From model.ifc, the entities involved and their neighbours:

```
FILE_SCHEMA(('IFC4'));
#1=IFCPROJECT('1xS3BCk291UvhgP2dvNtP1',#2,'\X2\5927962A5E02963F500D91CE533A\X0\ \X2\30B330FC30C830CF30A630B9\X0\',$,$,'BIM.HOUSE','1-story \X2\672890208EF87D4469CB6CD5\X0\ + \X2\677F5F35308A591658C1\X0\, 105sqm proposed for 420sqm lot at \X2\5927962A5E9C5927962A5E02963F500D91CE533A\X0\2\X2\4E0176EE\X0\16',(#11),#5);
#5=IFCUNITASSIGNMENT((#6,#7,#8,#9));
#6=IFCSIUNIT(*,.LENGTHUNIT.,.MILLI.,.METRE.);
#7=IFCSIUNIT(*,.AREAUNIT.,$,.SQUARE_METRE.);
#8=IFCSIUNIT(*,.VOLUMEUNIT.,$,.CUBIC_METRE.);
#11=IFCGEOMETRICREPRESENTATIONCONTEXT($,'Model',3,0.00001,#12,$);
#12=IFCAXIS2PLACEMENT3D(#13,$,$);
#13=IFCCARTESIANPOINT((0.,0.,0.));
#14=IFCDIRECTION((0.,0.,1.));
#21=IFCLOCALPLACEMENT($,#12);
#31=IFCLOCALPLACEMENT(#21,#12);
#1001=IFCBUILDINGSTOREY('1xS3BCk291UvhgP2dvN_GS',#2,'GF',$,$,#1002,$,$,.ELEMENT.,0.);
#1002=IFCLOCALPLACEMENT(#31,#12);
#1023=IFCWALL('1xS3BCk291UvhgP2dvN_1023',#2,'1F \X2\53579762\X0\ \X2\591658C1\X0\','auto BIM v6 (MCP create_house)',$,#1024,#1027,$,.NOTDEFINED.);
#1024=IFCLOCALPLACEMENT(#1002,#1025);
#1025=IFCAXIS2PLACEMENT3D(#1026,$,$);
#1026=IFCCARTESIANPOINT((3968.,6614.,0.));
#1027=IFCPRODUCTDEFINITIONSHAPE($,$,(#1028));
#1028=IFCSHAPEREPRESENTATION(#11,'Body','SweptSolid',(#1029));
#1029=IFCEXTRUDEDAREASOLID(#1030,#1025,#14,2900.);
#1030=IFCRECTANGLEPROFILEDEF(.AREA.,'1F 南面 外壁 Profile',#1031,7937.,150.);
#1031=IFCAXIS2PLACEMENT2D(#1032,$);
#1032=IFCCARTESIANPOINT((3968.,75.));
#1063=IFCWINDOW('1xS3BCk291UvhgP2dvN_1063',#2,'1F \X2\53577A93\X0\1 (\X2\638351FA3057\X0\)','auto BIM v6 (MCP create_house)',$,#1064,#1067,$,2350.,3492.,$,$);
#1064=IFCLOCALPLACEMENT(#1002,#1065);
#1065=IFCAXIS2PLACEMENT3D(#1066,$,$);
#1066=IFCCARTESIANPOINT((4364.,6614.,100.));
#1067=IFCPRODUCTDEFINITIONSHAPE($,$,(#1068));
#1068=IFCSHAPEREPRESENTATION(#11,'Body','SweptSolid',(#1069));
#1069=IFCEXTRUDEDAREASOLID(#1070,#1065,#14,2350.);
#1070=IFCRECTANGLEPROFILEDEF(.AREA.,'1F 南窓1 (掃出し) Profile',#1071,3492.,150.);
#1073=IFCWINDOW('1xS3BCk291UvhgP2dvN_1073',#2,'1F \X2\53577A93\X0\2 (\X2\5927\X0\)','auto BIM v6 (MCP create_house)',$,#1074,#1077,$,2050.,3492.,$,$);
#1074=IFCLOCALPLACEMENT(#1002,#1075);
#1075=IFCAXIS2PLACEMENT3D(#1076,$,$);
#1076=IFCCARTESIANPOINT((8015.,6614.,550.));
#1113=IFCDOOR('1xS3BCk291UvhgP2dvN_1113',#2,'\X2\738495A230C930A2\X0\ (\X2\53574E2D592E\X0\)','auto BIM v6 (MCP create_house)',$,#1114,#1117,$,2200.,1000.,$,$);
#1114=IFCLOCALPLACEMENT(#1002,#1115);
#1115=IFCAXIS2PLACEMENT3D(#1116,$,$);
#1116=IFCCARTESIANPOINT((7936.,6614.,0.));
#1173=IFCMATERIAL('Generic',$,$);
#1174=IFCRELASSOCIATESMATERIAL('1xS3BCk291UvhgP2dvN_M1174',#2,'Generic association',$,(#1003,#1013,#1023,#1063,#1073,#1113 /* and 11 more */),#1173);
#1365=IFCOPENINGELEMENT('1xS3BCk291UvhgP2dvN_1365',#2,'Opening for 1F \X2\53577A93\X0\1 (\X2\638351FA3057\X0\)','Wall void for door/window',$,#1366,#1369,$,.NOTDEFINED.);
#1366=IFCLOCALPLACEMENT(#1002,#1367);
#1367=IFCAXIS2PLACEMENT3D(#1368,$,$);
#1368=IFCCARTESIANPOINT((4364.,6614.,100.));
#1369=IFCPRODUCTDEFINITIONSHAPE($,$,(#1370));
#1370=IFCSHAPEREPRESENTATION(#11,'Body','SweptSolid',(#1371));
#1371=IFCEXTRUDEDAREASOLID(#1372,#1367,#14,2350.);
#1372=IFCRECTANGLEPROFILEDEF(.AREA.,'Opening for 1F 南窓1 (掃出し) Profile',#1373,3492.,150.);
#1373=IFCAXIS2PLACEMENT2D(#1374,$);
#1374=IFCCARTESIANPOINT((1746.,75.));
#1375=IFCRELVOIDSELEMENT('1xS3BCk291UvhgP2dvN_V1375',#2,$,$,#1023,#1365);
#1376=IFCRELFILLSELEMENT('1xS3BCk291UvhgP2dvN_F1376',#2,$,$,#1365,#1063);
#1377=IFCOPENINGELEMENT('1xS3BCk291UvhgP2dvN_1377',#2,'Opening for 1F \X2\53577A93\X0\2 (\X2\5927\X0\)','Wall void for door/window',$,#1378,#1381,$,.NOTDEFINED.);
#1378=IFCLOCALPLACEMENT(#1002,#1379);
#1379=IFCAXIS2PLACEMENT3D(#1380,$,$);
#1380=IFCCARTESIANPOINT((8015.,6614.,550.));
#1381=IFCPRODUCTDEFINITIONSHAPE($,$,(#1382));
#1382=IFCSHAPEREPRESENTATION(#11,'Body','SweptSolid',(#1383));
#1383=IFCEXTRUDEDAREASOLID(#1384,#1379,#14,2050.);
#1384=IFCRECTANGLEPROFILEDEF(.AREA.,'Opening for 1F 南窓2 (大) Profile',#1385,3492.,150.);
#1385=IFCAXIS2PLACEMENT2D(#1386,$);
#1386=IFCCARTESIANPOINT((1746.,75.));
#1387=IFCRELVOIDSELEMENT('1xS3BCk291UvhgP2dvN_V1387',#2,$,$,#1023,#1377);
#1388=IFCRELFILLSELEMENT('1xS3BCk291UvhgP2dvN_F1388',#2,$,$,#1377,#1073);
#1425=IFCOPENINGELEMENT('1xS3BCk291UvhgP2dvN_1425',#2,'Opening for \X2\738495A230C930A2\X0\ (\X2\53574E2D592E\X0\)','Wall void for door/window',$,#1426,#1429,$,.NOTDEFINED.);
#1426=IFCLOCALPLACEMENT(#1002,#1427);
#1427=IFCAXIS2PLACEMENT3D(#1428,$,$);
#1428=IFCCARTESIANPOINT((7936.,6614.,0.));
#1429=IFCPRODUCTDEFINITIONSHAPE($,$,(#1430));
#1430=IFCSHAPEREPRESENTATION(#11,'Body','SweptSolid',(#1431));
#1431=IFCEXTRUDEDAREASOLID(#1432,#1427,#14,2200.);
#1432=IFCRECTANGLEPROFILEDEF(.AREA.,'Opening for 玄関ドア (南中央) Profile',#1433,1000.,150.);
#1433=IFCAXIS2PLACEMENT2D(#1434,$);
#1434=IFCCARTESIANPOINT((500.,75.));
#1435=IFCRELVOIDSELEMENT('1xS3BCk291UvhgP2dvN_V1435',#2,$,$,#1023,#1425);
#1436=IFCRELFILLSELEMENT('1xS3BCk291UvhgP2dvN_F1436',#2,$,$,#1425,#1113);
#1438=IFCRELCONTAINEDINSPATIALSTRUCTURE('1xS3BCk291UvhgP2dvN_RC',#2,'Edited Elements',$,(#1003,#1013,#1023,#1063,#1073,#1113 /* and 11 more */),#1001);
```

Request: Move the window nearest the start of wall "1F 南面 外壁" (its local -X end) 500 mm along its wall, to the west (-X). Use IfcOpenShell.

```python
import ifcopenshell
import ifcopenshell.api.geometry
import ifcopenshell.util.placement
import ifcopenshell.util.unit

model = ifcopenshell.open("model.ifc")
unit_scale = ifcopenshell.util.unit.calculate_unit_scale(model)

window = model.by_guid("1xS3BCk291UvhgP2dvN_1063")
opening = window.FillsVoids[0].RelatingOpeningElement
wall = opening.VoidsElements[0].RelatingBuildingElement

wall_matrix = ifcopenshell.util.placement.get_local_placement(wall.ObjectPlacement)
shift = wall_matrix[:3, 0] * -0.5 / unit_scale
before = ifcopenshell.util.placement.get_local_placement(window.ObjectPlacement)[:3, 3].copy()

# The window is not placed relative to its opening, so move both.
for product in (opening, window):
    matrix = ifcopenshell.util.placement.get_local_placement(product.ObjectPlacement)
    matrix[:3, 3] += shift
    ifcopenshell.api.geometry.edit_object_placement(model, product=product, matrix=matrix, is_si=False)

after = ifcopenshell.util.placement.get_local_placement(window.ObjectPlacement)[:3, 3]
print("window moved by", (after - before).round(3) + 0.0)

model.write("model_v2.ifc")
```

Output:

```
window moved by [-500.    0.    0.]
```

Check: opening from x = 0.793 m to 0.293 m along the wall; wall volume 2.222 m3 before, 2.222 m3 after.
